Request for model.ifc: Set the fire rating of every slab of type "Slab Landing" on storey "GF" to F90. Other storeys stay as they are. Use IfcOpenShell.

First a look at what the model holds.

```python
import ifcopenshell
import ifcopenshell.util.element

model = ifcopenshell.open("model.ifc")
print(model.schema)
storey = next(s for s in model.by_type("IfcBuildingStorey") if s.Name == "GF")
slabs = [e for e in ifcopenshell.util.element.get_decomposition(storey) if e.is_a("IfcSlab")]
seen = {}
for e in slabs:
    element_type = ifcopenshell.util.element.get_type(e)
    key = (element_type.Name if element_type != e and element_type else None, ifcopenshell.util.element.get_pset(e, "Pset_SlabCommon", "FireRating"))
    seen[key] = seen.get(key, 0) + 1
for (name, value), count in sorted(seen.items(), key=str):
    print(count, "x", name, "|", value)
```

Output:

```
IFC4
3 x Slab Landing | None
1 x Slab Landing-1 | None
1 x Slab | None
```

```python
import ifcopenshell
import ifcopenshell.api.pset
import ifcopenshell.util.element

model = ifcopenshell.open("model.ifc")

storey = next(s for s in model.by_type("IfcBuildingStorey") if s.Name == "GF")
slabs = [e for e in ifcopenshell.util.element.get_decomposition(storey) if e.is_a("IfcSlab")]

count = 0
for e in slabs:
    element_type = ifcopenshell.util.element.get_type(e)
    if element_type in (None, e) or element_type.Name != "Slab Landing":
        continue
    # add_pset returns the element's existing set when there is one.
    pset = ifcopenshell.api.pset.add_pset(model, product=e, name="Pset_SlabCommon")
    ifcopenshell.api.pset.edit_pset(model, pset=pset, properties={"FireRating": "F90"})
    count += 1

print(count, "slabs updated")

model.write("model_edited.ifc")
```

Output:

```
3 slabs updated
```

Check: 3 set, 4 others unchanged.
